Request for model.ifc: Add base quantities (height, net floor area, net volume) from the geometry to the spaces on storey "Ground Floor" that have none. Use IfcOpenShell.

First a look at what the model holds.

```python
import ifcopenshell
import ifcopenshell.util.element
import ifcopenshell.util.unit

model = ifcopenshell.open("model.ifc")
print(model.schema)
for unit_type in ("LENGTHUNIT", "AREAUNIT", "VOLUMEUNIT"):
    print(unit_type, ifcopenshell.util.unit.calculate_unit_scale(model, unit_type))
storey = next(s for s in model.by_type("IfcBuildingStorey") if s.Name == "Ground Floor")
spaces = [e for e in ifcopenshell.util.element.get_decomposition(storey) if e.is_a("IfcSpace")]
for e in sorted(spaces, key=lambda e: e.id()):
    print(e.id(), e.is_a(), e.Name, list(ifcopenshell.util.element.get_psets(e, qtos_only=True)), sep=" | ")
```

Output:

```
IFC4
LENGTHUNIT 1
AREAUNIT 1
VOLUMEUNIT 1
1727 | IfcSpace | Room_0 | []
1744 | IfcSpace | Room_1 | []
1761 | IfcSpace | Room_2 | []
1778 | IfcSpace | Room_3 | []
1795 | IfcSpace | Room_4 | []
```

```python
import ifcopenshell
import ifcopenshell.api.pset
import ifcopenshell.geom
import ifcopenshell.util.element
import ifcopenshell.util.shape
import ifcopenshell.util.unit

model = ifcopenshell.open("model.ifc")
unit_scale = ifcopenshell.util.unit.calculate_unit_scale(model)
area_scale = ifcopenshell.util.unit.calculate_unit_scale(model, "AREAUNIT")
volume_scale = ifcopenshell.util.unit.calculate_unit_scale(model, "VOLUMEUNIT")
settings = ifcopenshell.geom.settings()

storey = next(s for s in model.by_type("IfcBuildingStorey") if s.Name == "Ground Floor")
spaces = [e for e in ifcopenshell.util.element.get_decomposition(storey) if e.is_a("IfcSpace")]

for e in sorted(spaces, key=lambda e: e.id()):
    if ifcopenshell.util.element.get_psets(e, qtos_only=True, should_inherit=False):
        continue
    # Geometry comes back in metres, in the element's own axes.
    shape = ifcopenshell.geom.create_shape(settings, e)
    values = {
        "Height": ifcopenshell.util.shape.get_z(shape.geometry) / unit_scale,
        "NetFloorArea": ifcopenshell.util.shape.get_footprint_area(shape.geometry) / area_scale,
        "NetVolume": ifcopenshell.util.shape.get_volume(shape.geometry) / volume_scale,
    }
    qto = ifcopenshell.api.pset.add_qto(model, product=e, name="Qto_SpaceBaseQuantities")
    ifcopenshell.api.pset.edit_qto(model, qto=qto, properties=values)
    print(e.id(), {k: round(v, 3) for k, v in values.items()})

model.write("model_edited.ifc")
```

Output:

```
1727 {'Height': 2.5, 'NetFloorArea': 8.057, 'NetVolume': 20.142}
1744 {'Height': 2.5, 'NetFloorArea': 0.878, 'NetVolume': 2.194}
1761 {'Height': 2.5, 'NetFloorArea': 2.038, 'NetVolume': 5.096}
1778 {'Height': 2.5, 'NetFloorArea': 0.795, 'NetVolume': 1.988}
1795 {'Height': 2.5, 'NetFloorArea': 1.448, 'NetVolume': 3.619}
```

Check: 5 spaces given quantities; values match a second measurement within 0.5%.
